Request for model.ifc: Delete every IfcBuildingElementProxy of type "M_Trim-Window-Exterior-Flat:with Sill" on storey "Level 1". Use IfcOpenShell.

First a look at what the model holds.

```python
import ifcopenshell
import ifcopenshell.util.element

model = ifcopenshell.open("model.ifc")
print(model.schema)
storey = next(s for s in model.by_type("IfcBuildingStorey") if s.Name == "Level 1")
proxies = [e for e in ifcopenshell.util.element.get_decomposition(storey) if e.is_a("IfcBuildingElementProxy")]
seen = {}
for e in proxies:
    element_type = ifcopenshell.util.element.get_type(e)
    name = element_type.Name if element_type not in (None, e) else None
    seen[name] = seen.get(name, 0) + 1
for name, count in sorted(seen.items(), key=str):
    print(count, "x", name)
```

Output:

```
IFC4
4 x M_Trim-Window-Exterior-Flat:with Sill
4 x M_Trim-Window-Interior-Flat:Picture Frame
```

```python
import ifcopenshell
import ifcopenshell.api.root
import ifcopenshell.util.element

model = ifcopenshell.open("model.ifc")

storey = next(s for s in model.by_type("IfcBuildingStorey") if s.Name == "Level 1")
proxies = [e for e in ifcopenshell.util.element.get_decomposition(storey) if e.is_a("IfcBuildingElementProxy")]
targets = [e for e in proxies if (t := ifcopenshell.util.element.get_type(e)) not in (None, e) and t.Name == "M_Trim-Window-Exterior-Flat:with Sill"]

for e in targets:
    ifcopenshell.api.root.remove_product(model, product=e)
print(len(targets), "removed")

model.write("model_v2.ifc")
```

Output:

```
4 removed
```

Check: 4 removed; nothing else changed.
